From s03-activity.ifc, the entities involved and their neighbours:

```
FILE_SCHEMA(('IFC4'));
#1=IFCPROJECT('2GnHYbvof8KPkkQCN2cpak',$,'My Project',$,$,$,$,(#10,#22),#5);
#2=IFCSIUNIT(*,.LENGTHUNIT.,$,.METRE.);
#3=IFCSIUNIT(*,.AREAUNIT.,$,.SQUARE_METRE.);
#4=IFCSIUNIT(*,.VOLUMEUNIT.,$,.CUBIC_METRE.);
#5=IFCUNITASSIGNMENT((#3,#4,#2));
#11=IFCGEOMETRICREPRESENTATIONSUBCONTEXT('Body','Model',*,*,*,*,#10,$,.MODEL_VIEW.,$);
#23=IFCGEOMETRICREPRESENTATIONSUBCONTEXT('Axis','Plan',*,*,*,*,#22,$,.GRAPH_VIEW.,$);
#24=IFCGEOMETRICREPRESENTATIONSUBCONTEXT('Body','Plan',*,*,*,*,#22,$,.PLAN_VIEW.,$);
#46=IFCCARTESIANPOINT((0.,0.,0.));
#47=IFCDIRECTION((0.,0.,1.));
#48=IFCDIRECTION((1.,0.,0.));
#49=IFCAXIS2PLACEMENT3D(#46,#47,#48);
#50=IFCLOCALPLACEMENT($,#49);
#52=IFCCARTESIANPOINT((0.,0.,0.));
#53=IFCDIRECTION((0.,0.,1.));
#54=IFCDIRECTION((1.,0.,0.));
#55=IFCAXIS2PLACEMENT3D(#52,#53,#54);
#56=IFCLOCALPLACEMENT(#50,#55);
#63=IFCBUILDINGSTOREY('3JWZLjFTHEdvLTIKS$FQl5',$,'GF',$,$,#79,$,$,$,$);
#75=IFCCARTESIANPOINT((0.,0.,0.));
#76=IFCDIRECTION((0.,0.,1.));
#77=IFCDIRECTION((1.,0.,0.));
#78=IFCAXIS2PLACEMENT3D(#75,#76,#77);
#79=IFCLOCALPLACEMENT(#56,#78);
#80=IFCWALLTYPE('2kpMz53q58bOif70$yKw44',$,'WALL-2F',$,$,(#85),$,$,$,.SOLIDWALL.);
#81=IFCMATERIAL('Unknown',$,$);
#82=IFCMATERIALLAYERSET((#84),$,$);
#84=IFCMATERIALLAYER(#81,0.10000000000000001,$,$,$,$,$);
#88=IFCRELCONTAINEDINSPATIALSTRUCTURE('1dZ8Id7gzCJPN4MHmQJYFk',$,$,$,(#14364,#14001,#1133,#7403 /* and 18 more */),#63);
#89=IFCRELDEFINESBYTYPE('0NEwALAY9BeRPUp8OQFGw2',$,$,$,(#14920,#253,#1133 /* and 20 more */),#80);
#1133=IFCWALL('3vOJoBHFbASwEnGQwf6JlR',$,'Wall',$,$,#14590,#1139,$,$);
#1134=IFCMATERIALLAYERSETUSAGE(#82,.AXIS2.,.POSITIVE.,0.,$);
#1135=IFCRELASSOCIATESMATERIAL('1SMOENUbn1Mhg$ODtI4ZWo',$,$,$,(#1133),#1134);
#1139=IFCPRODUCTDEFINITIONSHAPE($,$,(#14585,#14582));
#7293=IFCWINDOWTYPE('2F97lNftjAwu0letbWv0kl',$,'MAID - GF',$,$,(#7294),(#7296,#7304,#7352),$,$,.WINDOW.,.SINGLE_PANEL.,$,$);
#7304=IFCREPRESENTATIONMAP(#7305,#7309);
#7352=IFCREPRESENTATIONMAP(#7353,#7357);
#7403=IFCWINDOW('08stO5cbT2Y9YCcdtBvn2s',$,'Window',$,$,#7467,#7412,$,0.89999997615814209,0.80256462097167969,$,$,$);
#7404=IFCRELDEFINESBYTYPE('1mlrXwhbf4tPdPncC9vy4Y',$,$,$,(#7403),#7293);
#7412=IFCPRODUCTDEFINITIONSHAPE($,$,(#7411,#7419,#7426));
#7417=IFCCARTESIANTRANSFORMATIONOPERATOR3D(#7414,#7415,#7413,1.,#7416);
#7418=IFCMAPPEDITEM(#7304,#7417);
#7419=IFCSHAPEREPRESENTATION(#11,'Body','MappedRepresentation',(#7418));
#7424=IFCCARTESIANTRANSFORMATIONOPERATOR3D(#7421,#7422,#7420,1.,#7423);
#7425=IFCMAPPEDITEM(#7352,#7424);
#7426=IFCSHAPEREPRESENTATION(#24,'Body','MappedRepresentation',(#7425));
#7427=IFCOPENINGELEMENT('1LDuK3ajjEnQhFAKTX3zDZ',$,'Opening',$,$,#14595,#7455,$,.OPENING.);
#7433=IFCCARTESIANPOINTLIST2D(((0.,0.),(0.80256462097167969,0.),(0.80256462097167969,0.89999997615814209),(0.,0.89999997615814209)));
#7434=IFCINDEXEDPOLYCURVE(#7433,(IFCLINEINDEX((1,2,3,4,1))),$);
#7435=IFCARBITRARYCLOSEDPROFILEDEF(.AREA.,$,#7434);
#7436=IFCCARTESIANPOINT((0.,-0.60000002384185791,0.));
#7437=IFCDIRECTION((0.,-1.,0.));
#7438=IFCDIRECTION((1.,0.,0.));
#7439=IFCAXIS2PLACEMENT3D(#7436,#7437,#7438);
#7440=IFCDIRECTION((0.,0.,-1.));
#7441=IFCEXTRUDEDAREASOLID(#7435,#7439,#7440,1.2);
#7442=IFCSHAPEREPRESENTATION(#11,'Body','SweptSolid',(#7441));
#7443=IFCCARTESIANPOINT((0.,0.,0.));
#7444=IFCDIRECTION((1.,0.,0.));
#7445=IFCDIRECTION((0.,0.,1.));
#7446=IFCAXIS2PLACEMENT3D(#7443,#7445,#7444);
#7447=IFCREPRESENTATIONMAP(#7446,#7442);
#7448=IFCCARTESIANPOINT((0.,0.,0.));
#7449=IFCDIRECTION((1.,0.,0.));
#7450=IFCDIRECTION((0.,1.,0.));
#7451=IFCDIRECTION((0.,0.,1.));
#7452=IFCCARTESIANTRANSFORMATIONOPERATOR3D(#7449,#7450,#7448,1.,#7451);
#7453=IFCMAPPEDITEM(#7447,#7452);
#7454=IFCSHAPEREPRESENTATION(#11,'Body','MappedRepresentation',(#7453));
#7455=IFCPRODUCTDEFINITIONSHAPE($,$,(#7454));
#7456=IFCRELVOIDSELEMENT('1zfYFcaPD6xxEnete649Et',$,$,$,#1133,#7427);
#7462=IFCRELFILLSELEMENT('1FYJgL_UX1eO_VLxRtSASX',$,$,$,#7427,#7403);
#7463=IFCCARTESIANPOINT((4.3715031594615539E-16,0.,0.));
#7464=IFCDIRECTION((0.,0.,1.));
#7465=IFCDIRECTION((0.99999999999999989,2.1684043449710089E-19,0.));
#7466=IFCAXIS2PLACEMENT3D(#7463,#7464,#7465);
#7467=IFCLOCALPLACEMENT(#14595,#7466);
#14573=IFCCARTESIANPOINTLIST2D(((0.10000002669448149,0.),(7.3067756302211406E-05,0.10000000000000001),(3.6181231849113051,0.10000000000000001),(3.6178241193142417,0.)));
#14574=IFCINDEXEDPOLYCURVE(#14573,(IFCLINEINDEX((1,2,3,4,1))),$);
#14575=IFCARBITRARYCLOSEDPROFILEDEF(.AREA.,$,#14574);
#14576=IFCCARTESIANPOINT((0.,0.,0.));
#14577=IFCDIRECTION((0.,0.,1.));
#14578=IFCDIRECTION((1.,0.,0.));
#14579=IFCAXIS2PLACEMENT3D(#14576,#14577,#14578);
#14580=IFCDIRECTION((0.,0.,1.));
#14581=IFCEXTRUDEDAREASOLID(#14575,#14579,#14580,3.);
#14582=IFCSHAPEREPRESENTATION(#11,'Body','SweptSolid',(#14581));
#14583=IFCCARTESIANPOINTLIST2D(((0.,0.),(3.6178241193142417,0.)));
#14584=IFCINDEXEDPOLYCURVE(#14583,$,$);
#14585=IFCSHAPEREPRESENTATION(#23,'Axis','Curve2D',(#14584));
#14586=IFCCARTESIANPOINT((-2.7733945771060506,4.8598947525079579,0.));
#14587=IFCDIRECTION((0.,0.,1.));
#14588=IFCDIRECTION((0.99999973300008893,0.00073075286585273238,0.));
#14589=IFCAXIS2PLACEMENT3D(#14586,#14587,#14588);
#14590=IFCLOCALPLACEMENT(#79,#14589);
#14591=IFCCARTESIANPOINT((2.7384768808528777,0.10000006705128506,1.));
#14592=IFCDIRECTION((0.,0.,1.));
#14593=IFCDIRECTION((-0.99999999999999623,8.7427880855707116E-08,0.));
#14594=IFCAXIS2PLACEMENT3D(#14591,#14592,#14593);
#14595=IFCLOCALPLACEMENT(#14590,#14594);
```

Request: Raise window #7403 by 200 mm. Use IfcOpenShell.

```python
import numpy as np
import ifcopenshell
import ifcopenshell.api.geometry
import ifcopenshell.util.placement
import ifcopenshell.util.unit

model = ifcopenshell.open("s03-activity.ifc")
unit_scale = ifcopenshell.util.unit.calculate_unit_scale(model)

window = model.by_guid("08stO5cbT2Y9YCcdtBvn2s")
opening = window.FillsVoids[0].RelatingOpeningElement
dz = 0.2 / unit_scale

shift = np.array([0.0, 0.0, dz])
# The window is placed relative to its opening, so it follows when the opening moves.
matrix = ifcopenshell.util.placement.get_local_placement(opening.ObjectPlacement)
matrix[:3, 3] += shift
ifcopenshell.api.geometry.edit_object_placement(
    model, product=opening, matrix=matrix, is_si=False, should_transform_children=True
)

print(f"moved by {dz * unit_scale:+.3f} m")

model.write("s03-activity_edited.ifc")
```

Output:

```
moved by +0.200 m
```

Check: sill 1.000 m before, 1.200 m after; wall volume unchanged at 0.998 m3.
